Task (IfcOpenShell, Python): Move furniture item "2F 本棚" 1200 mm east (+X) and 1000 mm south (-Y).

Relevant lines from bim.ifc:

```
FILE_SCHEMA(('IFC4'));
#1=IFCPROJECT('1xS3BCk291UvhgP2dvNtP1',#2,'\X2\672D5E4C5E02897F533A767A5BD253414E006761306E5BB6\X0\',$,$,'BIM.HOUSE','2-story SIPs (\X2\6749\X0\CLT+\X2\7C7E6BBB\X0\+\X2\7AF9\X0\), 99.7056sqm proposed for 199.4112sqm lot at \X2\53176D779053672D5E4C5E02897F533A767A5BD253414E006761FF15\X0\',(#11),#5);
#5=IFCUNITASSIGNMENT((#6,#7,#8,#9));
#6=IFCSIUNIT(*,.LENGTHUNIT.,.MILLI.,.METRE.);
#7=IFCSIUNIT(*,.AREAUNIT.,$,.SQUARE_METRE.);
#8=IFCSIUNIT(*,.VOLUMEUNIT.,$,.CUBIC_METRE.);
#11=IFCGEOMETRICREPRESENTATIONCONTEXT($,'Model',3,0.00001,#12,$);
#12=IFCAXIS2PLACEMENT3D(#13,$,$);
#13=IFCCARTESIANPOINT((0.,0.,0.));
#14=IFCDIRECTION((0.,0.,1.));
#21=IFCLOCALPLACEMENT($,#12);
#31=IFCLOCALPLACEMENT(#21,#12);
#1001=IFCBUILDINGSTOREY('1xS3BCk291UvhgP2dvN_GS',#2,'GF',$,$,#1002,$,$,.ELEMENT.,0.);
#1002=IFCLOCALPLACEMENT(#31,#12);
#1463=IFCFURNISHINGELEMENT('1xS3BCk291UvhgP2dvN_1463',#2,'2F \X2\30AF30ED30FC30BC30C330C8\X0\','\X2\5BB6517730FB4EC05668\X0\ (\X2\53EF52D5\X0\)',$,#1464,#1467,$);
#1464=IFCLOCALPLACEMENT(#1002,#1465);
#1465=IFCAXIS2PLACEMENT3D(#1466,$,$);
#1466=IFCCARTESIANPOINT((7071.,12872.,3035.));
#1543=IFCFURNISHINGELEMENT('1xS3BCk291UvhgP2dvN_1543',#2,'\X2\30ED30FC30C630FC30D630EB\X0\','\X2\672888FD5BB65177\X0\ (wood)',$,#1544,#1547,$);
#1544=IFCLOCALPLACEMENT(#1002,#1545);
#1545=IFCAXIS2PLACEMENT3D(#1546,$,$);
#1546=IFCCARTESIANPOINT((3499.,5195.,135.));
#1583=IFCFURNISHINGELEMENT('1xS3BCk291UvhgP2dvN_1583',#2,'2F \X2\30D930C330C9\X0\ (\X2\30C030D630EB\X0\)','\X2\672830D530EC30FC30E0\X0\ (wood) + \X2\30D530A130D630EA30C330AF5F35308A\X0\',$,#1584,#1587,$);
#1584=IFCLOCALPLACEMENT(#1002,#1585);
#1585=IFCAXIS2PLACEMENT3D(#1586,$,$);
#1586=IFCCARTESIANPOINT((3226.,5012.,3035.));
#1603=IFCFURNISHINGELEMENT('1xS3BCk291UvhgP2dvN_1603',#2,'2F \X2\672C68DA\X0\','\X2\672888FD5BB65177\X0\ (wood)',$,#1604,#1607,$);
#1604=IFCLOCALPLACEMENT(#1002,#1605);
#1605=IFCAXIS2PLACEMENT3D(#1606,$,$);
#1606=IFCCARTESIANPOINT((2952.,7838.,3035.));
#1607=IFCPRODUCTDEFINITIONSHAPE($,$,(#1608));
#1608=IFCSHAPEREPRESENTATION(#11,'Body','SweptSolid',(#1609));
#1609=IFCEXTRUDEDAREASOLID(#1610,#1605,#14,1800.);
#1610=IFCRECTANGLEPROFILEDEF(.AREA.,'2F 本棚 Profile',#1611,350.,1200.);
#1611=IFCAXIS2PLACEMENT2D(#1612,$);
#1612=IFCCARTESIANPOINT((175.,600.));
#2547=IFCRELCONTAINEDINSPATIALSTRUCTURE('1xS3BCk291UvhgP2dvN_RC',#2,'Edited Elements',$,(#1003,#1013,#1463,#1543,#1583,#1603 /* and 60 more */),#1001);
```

```python
import ifcopenshell
import ifcopenshell.api.geometry
import ifcopenshell.util.placement

model = ifcopenshell.open("bim.ifc")

item = model.by_guid("1xS3BCk291UvhgP2dvN_1603")
matrix = ifcopenshell.util.placement.get_local_placement(item.ObjectPlacement)
matrix[0, 3] += 1200.0
matrix[1, 3] -= 1000.0
ifcopenshell.api.geometry.edit_object_placement(model, product=item, matrix=matrix, is_si=False)

print(ifcopenshell.util.placement.get_local_placement(item.ObjectPlacement).round(3) + 0.0)

model.write("bim_rev.ifc")
```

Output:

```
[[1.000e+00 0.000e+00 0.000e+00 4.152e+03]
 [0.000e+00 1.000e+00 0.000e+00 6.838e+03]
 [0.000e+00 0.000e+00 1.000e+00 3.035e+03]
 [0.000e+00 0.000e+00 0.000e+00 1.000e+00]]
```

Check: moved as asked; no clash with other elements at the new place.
